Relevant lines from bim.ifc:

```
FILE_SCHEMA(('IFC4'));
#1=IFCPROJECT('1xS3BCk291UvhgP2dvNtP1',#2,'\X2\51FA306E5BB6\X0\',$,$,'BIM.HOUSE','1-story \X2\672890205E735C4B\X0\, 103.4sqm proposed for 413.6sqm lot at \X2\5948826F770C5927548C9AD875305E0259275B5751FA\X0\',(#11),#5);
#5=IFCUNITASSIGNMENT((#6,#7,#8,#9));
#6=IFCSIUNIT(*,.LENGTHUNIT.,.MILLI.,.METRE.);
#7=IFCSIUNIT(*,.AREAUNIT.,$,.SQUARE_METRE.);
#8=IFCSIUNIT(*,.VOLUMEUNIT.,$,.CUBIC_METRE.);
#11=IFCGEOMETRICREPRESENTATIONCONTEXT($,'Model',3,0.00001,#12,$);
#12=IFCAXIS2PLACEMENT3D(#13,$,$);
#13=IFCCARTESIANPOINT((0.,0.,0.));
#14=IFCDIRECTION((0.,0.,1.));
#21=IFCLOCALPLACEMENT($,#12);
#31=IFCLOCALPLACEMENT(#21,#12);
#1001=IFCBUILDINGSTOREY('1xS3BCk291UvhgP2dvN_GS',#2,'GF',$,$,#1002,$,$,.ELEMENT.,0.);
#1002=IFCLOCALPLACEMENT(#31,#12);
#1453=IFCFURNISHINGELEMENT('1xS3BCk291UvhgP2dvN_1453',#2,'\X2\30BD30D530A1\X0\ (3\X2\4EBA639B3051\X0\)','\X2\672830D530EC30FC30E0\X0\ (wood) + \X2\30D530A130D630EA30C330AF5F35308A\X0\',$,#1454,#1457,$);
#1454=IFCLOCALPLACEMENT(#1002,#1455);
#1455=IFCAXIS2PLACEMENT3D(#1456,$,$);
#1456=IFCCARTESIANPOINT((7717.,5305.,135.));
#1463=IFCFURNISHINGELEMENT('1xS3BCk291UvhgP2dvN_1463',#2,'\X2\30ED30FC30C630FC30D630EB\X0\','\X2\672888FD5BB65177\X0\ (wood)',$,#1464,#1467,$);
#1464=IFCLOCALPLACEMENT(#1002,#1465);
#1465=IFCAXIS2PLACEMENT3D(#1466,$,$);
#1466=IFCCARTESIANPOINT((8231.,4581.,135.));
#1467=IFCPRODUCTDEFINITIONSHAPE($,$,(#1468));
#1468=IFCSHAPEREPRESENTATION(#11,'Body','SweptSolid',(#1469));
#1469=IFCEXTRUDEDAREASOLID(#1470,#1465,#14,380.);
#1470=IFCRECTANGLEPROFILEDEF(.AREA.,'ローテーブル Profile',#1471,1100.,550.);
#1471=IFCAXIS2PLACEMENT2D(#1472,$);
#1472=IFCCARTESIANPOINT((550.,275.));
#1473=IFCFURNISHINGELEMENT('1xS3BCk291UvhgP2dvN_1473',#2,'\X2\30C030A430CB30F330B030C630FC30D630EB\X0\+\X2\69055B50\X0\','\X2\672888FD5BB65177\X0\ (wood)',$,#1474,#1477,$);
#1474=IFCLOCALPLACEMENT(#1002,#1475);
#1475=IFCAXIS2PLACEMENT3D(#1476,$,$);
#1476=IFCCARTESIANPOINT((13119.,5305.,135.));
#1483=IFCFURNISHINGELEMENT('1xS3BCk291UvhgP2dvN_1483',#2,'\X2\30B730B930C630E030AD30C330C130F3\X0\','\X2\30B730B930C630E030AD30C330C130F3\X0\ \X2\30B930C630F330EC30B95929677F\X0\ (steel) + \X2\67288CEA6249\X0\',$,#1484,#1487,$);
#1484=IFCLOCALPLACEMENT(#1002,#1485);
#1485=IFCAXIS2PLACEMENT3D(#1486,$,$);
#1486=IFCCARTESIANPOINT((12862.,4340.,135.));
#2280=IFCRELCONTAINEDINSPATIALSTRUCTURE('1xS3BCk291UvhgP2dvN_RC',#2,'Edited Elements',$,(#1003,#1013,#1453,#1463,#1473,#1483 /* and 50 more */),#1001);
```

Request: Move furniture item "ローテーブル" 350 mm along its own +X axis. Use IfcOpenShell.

```python
import ifcopenshell
import ifcopenshell.api.geometry
import ifcopenshell.util.placement

model = ifcopenshell.open("bim.ifc")

item = model.by_id(1463)
matrix = ifcopenshell.util.placement.get_local_placement(item.ObjectPlacement)
matrix[:3, 3] += matrix[:3, 0] * 350.0
ifcopenshell.api.geometry.edit_object_placement(model, product=item, matrix=matrix, is_si=False)

print(ifcopenshell.util.placement.get_local_placement(item.ObjectPlacement).round(3) + 0.0)

model.write("bim_updated.ifc")
```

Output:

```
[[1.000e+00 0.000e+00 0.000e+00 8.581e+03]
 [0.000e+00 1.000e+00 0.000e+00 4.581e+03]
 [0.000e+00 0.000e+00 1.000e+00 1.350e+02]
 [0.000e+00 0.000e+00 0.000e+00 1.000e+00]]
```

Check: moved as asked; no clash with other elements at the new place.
